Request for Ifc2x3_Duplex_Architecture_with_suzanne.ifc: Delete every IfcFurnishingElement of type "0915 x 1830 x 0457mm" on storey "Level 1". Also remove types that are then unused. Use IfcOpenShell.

First a look at what the model holds.

```python
import ifcopenshell
import ifcopenshell.util.element

model = ifcopenshell.open("Ifc2x3_Duplex_Architecture_with_suzanne.ifc")
print(model.schema)
storey = next(s for s in model.by_type("IfcBuildingStorey") if s.Name == "Level 1")
furniture = [e for e in ifcopenshell.util.element.get_decomposition(storey) if e.is_a("IfcFurnishingElement")]
seen = {}
for e in furniture:
    element_type = ifcopenshell.util.element.get_type(e)
    name = element_type.Name if element_type not in (None, e) else None
    seen[name] = seen.get(name, 0) + 1
for name, count in sorted(seen.items(), key=str):
    print(count, "x", name)
```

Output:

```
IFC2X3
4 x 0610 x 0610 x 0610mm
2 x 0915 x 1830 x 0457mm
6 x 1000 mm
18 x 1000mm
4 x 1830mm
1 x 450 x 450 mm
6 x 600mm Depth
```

```python
import ifcopenshell
import ifcopenshell.api.root
import ifcopenshell.util.element

model = ifcopenshell.open("Ifc2x3_Duplex_Architecture_with_suzanne.ifc")

storey = next(s for s in model.by_type("IfcBuildingStorey") if s.Name == "Level 1")
furniture = [e for e in ifcopenshell.util.element.get_decomposition(storey) if e.is_a("IfcFurnishingElement")]
targets = [e for e in furniture if (t := ifcopenshell.util.element.get_type(e)) not in (None, e) and t.Name == "0915 x 1830 x 0457mm"]
types = {ifcopenshell.util.element.get_type(e) for e in targets} - {None, *targets}

for e in targets:
    ifcopenshell.api.root.remove_product(model, product=e)
print(len(targets), "removed")

unused = [t for t in types if not ifcopenshell.util.element.get_types(t)]
for t in unused:
    ifcopenshell.api.root.remove_product(model, product=t)
print(len(unused), "unused types removed")

model.write("Ifc2x3_Duplex_Architecture_with_suzanne_rev.ifc")
```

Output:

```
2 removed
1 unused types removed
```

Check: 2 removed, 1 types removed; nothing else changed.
